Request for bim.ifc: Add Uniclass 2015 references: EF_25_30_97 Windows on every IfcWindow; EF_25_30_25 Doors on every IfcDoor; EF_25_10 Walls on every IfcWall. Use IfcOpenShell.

First a look at what the model holds.

```python
import ifcopenshell

model = ifcopenshell.open("bim.ifc")
print(model.schema)
print("classifications:", [c.Name for c in model.by_type("IfcClassification")])
for ifc_class in ("IfcDoor", "IfcRoof", "IfcStair", "IfcWall", "IfcWindow"):
    print(ifc_class, len(model.by_type(ifc_class)))
```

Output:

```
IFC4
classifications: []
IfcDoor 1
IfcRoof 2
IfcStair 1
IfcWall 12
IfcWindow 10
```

```python
import ifcopenshell
import ifcopenshell.api.classification

model = ifcopenshell.open("bim.ifc")

system = ifcopenshell.api.classification.add_classification(model, classification="Uniclass 2015")

codes = {
    "IfcWindow": ("EF_25_30_97", "Windows"),
    "IfcDoor": ("EF_25_30_25", "Doors"),
    "IfcWall": ("EF_25_10", "Walls"),
}
for ifc_class, (code, name) in codes.items():
    products = model.by_type(ifc_class)
    ifcopenshell.api.classification.add_reference(
        model, products=products, classification=system, identification=code, name=name
    )
    print(code, len(products))

model.write("bim_updated.ifc")
```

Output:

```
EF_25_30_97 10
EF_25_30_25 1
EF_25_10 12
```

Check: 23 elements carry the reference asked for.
